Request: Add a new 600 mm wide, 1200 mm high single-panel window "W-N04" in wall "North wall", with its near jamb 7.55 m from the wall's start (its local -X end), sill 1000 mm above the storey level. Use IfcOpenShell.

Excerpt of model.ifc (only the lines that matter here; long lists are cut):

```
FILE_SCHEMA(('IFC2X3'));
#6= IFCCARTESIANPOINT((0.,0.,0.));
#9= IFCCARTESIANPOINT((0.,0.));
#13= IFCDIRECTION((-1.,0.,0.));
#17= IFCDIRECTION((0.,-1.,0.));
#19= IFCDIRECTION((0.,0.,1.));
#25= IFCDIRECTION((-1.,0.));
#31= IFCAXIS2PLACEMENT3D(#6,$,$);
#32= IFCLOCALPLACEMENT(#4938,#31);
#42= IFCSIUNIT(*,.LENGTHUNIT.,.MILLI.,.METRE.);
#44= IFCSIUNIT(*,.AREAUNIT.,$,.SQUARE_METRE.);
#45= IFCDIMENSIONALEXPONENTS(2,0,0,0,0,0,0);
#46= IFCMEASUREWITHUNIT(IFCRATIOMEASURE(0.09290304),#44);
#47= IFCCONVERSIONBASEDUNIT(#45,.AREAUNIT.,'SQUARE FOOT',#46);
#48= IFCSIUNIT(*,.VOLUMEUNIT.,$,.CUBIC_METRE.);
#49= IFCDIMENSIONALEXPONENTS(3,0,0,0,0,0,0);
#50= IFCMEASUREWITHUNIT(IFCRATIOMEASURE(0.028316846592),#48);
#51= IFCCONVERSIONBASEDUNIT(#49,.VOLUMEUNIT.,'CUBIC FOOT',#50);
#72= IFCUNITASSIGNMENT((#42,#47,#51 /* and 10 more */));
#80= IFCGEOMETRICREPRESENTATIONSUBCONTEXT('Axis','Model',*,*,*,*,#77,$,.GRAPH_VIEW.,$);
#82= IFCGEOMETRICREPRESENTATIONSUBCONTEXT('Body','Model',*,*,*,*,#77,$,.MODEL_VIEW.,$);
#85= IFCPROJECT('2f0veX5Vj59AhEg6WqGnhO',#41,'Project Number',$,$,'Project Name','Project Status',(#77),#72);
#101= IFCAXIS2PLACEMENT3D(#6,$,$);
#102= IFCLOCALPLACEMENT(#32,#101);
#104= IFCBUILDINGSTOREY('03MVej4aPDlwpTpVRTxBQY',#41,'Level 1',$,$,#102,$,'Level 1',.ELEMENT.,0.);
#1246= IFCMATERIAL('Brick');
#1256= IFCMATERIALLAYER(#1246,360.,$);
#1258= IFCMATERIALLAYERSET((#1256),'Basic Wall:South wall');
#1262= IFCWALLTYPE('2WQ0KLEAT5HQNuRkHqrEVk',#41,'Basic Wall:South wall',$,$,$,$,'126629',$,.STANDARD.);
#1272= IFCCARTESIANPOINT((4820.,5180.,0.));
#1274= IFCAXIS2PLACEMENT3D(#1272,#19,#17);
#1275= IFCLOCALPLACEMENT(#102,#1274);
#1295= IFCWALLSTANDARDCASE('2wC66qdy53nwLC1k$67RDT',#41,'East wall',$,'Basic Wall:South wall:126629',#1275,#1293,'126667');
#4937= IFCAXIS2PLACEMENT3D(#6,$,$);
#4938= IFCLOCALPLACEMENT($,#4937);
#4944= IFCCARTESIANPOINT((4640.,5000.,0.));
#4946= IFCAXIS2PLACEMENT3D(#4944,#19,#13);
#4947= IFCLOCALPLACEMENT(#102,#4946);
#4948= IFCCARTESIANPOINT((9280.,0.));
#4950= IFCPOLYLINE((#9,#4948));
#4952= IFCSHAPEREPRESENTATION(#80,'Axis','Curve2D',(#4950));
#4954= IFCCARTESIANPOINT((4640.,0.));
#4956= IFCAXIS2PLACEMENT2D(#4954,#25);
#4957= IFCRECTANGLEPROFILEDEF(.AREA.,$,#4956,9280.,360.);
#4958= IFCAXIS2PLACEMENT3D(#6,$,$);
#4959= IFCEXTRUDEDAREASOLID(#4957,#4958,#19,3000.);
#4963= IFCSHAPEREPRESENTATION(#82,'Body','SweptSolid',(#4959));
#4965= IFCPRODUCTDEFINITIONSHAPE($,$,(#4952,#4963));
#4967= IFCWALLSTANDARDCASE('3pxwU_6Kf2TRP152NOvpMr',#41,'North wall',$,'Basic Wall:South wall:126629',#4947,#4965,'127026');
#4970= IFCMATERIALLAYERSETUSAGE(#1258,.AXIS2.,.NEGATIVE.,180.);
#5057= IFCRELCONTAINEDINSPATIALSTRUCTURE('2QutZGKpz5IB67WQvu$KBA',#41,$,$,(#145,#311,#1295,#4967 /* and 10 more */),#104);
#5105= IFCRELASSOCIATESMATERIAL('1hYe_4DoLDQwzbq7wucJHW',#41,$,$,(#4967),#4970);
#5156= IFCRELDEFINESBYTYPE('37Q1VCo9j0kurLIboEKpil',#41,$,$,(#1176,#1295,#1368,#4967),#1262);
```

```python
import numpy as np
import ifcopenshell
import ifcopenshell.api.feature
import ifcopenshell.api.geometry
import ifcopenshell.api.root
import ifcopenshell.api.spatial
import ifcopenshell.api.type
import ifcopenshell.geom
import ifcopenshell.util.element
import ifcopenshell.util.placement
import ifcopenshell.util.representation
import ifcopenshell.util.shape
import ifcopenshell.util.unit

model = ifcopenshell.open("model.ifc")
unit_scale = ifcopenshell.util.unit.calculate_unit_scale(model)
settings = ifcopenshell.geom.settings()


def volume(element):
    """Net volume in cubic metres, openings subtracted."""
    shape = ifcopenshell.geom.create_shape(settings, element)
    return ifcopenshell.util.shape.get_volume(shape.geometry)


wall = model.by_guid("3pxwU_6Kf2TRP152NOvpMr")
storey = ifcopenshell.util.element.get_container(wall, ifc_class="IfcBuildingStorey")
context = ifcopenshell.util.representation.get_context(model, "Model", "Body", "MODEL_VIEW")
before = volume(wall)

width, height, from_end, sill = 0.6, 1.2, 7.55, 1  # metres

# The wall runs along its own X axis, and the end named is its -X end.
wall_shape = ifcopenshell.geom.create_shape(settings, wall)
x, y, z = ifcopenshell.util.shape.get_vertices(wall_shape.geometry).T
start = x.min() + from_end
face, thickness = float(y.min()), float(y.max() - y.min())
wall_matrix = ifcopenshell.util.placement.get_local_placement(wall.ObjectPlacement)
level = ifcopenshell.util.placement.get_local_placement(storey.ObjectPlacement)[2, 3]


def in_wall(x, y):
    """Placement at x, y metres in the wall's axes, at sill height."""
    matrix = wall_matrix.copy()
    matrix[:, 3] = wall_matrix @ np.array([x / unit_scale, y / unit_scale, 0.0, 1.0])
    matrix[2, 3] = level + sill / unit_scale
    return matrix


# Opening: a box that overshoots both wall faces by 50 mm.
opening = ifcopenshell.api.root.create_entity(model, ifc_class="IfcOpeningElement")
box = ifcopenshell.api.geometry.add_wall_representation(
    model, context=context, length=width, height=height, thickness=thickness + 0.1
)
ifcopenshell.api.geometry.assign_representation(model, product=opening, representation=box)
ifcopenshell.api.geometry.edit_object_placement(model, product=opening, matrix=in_wall(start, face - 0.05), is_si=False)
ifcopenshell.api.feature.add_feature(model, feature=opening, element=wall)

window = ifcopenshell.api.root.create_entity(model, ifc_class="IfcWindow", name="W-N04")
window.OverallWidth, window.OverallHeight = width / unit_scale, height / unit_scale
body = ifcopenshell.api.geometry.add_window_representation(
    model,
    context=context,
    overall_width=window.OverallWidth,
    overall_height=window.OverallHeight,
    partition_type="SINGLE_PANEL",
)
ifcopenshell.api.geometry.assign_representation(model, product=window, representation=body)
ifcopenshell.api.spatial.assign_container(model, products=[window], relating_structure=storey)
fills = ifcopenshell.api.feature.add_filling(model, opening=opening, element=window)
fills.OwnerHistory = window.OwnerHistory  # required in IFC2X3

# IFC2X3 keeps the operation on the window style.
style = ifcopenshell.api.root.create_entity(model, ifc_class="IfcWindowStyle", name="W-N04")
style.OperationType, style.ConstructionType = "SINGLE_PANEL", "NOTDEFINED"
style.ParameterTakesPrecedence = style.Sizeable = False
ifcopenshell.api.type.assign_type(model, related_objects=[window], relating_type=style)

# Centre the window in the wall's thickness.
ifcopenshell.api.geometry.edit_object_placement(model, product=window, matrix=in_wall(start, face), is_si=False)
window_shape = ifcopenshell.geom.create_shape(settings, window)
depth = ifcopenshell.util.shape.get_vertices(window_shape.geometry)[:, 1]
offset = face + thickness / 2 - (depth.min() + depth.max()) / 2
ifcopenshell.api.geometry.edit_object_placement(model, product=window, matrix=in_wall(start, offset), is_si=False)

after = volume(wall)

print(f"wall volume {before:.3f} -> {after:.3f} m3")

model.write("model_rev.ifc")
```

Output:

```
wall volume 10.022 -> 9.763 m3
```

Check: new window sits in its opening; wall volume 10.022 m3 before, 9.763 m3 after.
